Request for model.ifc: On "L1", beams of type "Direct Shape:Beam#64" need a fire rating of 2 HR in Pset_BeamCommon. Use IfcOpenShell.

First a look at what the model holds.

```python
import ifcopenshell
import ifcopenshell.util.element

model = ifcopenshell.open("model.ifc")
print(model.schema)
storey = next(s for s in model.by_type("IfcBuildingStorey") if s.Name == "L1")
beams = [e for e in ifcopenshell.util.element.get_decomposition(storey) if e.is_a("IfcBeam")]
seen = {}
for e in beams:
    element_type = ifcopenshell.util.element.get_type(e)
    key = (element_type.Name if element_type != e and element_type else None, ifcopenshell.util.element.get_pset(e, "Pset_BeamCommon", "FireRating"))
    seen[key] = seen.get(key, 0) + 1
for (name, value), count in sorted(seen.items(), key=str):
    print(count, "x", name, "|", value)
```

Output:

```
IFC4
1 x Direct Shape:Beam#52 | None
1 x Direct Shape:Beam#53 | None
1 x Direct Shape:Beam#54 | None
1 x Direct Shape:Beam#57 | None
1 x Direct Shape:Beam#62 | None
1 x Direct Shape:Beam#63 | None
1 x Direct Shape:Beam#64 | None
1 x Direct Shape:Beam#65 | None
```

```python
import ifcopenshell
import ifcopenshell.api.pset
import ifcopenshell.util.element

model = ifcopenshell.open("model.ifc")

storey = next(s for s in model.by_type("IfcBuildingStorey") if s.Name == "L1")
beams = [e for e in ifcopenshell.util.element.get_decomposition(storey) if e.is_a("IfcBeam")]

count = 0
for e in beams:
    element_type = ifcopenshell.util.element.get_type(e)
    if element_type in (None, e) or element_type.Name != "Direct Shape:Beam#64":
        continue
    # add_pset returns the element's existing set when there is one.
    pset = ifcopenshell.api.pset.add_pset(model, product=e, name="Pset_BeamCommon")
    ifcopenshell.api.pset.edit_pset(model, pset=pset, properties={"FireRating": "2 HR"})
    count += 1

print(count, "beams updated")

model.write("model_updated.ifc")
```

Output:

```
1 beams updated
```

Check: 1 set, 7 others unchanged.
